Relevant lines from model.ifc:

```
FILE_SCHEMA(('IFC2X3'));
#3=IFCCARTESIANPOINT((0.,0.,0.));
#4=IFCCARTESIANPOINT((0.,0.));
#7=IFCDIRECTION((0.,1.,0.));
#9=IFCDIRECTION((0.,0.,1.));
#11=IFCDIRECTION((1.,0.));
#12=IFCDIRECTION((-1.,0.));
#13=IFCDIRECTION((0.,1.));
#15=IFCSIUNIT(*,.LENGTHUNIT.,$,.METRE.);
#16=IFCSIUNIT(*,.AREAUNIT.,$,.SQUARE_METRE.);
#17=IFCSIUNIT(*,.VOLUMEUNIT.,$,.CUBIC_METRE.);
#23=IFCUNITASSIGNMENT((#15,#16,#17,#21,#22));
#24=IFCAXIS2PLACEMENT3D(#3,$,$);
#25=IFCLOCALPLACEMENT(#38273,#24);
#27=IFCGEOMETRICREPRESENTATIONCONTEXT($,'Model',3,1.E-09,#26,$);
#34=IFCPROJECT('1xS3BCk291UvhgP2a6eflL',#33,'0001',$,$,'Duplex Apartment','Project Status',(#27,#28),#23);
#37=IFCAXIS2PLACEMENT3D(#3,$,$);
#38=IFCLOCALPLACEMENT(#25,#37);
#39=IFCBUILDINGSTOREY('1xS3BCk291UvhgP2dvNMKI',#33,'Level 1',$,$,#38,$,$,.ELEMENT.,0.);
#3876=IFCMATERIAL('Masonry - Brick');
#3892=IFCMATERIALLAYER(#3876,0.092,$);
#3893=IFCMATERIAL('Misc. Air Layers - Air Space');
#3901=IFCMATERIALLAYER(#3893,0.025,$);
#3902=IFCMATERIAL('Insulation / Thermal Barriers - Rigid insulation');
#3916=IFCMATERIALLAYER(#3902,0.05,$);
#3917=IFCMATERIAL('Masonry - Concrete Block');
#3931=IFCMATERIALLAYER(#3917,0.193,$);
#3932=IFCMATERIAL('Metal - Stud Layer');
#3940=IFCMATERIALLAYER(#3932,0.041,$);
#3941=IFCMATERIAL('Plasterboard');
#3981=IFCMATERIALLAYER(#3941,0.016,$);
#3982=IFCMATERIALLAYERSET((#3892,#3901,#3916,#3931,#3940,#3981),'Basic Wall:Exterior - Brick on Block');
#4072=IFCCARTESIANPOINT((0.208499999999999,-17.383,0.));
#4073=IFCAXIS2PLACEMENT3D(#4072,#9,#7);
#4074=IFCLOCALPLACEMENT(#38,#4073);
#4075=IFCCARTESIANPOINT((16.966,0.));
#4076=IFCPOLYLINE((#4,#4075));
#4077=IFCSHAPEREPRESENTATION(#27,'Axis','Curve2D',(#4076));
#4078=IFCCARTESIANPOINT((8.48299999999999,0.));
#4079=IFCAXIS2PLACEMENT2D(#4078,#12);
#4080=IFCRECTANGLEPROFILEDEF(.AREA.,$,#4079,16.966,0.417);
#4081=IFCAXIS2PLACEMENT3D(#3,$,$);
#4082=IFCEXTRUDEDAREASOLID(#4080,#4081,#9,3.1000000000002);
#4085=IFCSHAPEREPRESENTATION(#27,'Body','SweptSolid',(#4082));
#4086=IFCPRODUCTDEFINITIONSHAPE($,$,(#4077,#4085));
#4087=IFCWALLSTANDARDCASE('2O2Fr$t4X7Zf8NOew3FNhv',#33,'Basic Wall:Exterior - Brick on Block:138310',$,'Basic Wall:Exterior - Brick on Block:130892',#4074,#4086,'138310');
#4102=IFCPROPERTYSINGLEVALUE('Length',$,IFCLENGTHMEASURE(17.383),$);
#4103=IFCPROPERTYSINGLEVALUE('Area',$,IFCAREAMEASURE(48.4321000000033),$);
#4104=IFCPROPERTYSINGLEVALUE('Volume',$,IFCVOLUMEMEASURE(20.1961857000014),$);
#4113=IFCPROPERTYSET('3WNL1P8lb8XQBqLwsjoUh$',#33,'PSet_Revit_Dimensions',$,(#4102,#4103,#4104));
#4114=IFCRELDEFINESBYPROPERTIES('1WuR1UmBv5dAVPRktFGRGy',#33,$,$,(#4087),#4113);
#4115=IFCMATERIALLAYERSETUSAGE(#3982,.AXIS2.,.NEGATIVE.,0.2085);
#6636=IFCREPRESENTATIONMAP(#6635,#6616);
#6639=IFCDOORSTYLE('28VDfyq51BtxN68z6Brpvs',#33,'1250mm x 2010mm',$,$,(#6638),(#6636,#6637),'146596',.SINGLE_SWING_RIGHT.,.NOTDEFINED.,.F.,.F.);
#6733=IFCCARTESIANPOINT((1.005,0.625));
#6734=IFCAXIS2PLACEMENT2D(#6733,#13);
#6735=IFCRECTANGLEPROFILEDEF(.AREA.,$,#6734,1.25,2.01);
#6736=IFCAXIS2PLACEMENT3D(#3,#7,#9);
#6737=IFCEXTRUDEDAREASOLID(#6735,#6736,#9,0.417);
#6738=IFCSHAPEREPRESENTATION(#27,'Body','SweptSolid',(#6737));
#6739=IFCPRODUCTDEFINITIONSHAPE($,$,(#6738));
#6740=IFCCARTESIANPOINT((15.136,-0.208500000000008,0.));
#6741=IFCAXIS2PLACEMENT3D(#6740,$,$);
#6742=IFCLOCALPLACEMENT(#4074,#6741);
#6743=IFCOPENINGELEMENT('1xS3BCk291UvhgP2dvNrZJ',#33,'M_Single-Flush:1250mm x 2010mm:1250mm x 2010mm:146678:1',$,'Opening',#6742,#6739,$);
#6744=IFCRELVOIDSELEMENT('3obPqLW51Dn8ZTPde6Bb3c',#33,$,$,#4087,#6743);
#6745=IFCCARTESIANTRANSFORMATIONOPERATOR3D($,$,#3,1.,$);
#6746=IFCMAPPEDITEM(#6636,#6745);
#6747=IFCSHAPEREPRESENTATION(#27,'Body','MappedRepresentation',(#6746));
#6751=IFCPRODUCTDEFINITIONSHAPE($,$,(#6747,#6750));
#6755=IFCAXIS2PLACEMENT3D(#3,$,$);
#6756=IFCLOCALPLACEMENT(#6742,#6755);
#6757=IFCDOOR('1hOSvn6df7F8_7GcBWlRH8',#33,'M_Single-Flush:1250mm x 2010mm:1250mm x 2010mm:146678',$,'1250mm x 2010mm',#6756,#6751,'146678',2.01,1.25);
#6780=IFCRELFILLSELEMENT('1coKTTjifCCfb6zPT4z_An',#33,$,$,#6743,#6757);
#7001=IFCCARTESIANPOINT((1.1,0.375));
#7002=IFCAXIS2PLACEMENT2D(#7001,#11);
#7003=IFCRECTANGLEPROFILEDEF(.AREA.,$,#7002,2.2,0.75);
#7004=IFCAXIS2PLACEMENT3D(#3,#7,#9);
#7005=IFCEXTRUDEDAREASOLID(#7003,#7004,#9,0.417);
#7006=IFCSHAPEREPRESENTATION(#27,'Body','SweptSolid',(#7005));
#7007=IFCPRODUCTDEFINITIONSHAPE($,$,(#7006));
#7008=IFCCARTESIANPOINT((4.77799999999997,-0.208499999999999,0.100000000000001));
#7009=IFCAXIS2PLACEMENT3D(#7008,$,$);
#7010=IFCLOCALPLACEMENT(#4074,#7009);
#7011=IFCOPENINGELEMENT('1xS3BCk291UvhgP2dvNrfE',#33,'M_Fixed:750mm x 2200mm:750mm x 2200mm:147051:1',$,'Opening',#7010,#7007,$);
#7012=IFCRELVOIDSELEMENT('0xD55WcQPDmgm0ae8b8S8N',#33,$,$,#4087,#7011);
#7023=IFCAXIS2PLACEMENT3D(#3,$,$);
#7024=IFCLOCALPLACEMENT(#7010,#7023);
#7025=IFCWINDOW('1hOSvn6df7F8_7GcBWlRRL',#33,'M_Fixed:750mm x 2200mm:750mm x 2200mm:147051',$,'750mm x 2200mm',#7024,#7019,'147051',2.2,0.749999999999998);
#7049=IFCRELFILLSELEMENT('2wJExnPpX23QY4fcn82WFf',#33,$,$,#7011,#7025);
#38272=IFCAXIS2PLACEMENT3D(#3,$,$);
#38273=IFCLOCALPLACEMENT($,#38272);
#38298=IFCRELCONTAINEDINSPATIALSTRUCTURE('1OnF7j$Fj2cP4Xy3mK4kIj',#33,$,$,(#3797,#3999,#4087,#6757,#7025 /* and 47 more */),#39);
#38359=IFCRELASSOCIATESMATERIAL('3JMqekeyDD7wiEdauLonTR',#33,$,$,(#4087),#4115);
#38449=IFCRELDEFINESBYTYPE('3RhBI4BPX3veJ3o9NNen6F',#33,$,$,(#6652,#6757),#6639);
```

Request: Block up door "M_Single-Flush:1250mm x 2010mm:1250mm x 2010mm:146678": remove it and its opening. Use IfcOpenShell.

```python
import ifcopenshell
import ifcopenshell.api.feature
import ifcopenshell.api.pset
import ifcopenshell.api.root
import ifcopenshell.geom
import ifcopenshell.util.element
import ifcopenshell.util.shape
import ifcopenshell.util.unit

model = ifcopenshell.open("model.ifc")
area_scale = ifcopenshell.util.unit.calculate_unit_scale(model, "AREAUNIT")
volume_scale = ifcopenshell.util.unit.calculate_unit_scale(model, "VOLUMEUNIT")
settings = ifcopenshell.geom.settings()


def volume(element):
    """Net volume in cubic metres, openings subtracted."""
    shape = ifcopenshell.geom.create_shape(settings, element)
    return ifcopenshell.util.shape.get_volume(shape.geometry)


door = model.by_guid("1hOSvn6df7F8_7GcBWlRH8")
opening = door.FillsVoids[0].RelatingOpeningElement
wall = opening.VoidsElements[0].RelatingBuildingElement
before = volume(wall)

ifcopenshell.api.root.remove_product(model, product=door)
ifcopenshell.api.feature.remove_feature(model, feature=opening)

after = volume(wall)
thickness = 0.417  # wall thickness in metres

# Update the wall's stored quantities.
pset = model.by_id(ifcopenshell.util.element.get_pset(wall, "PSet_Revit_Dimensions", should_inherit=False)["id"])
ifcopenshell.api.pset.edit_pset(model, pset=pset, properties={
    "Area": model.create_entity("IfcAreaMeasure", after / thickness / area_scale),
    "Volume": model.create_entity("IfcVolumeMeasure", after / volume_scale),
})

print(f"wall volume {before:.3f} -> {after:.3f} m3")

model.write("model_v2.ifc")
```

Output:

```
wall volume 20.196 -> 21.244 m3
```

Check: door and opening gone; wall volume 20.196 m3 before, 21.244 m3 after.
